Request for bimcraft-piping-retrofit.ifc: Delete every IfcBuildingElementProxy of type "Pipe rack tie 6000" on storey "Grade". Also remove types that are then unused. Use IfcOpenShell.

First a look at what the model holds.

```python
import ifcopenshell
import ifcopenshell.util.element

model = ifcopenshell.open("bimcraft-piping-retrofit.ifc")
print(model.schema)
storey = next(s for s in model.by_type("IfcBuildingStorey") if s.Name == "Grade")
proxies = [e for e in ifcopenshell.util.element.get_decomposition(storey) if e.is_a("IfcBuildingElementProxy")]
seen = {}
for e in proxies:
    element_type = ifcopenshell.util.element.get_type(e)
    name = element_type.Name if element_type not in (None, e) else None
    seen[name] = seen.get(name, 0) + 1
for name, count in sorted(seen.items(), key=str):
    print(count, "x", name)
```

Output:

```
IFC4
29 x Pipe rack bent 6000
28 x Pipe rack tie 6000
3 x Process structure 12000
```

```python
import ifcopenshell
import ifcopenshell.api.root
import ifcopenshell.util.element

model = ifcopenshell.open("bimcraft-piping-retrofit.ifc")

storey = next(s for s in model.by_type("IfcBuildingStorey") if s.Name == "Grade")
proxies = [e for e in ifcopenshell.util.element.get_decomposition(storey) if e.is_a("IfcBuildingElementProxy")]
targets = [e for e in proxies if (t := ifcopenshell.util.element.get_type(e)) not in (None, e) and t.Name == "Pipe rack tie 6000"]
types = {ifcopenshell.util.element.get_type(e) for e in targets} - {None, *targets}

for e in targets:
    ifcopenshell.api.root.remove_product(model, product=e)
print(len(targets), "removed")

unused = [t for t in types if not ifcopenshell.util.element.get_types(t)]
for t in unused:
    ifcopenshell.api.root.remove_product(model, product=t)
print(len(unused), "unused types removed")

model.write("bimcraft-piping-retrofit_rev.ifc")
```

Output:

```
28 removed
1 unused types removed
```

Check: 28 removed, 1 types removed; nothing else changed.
